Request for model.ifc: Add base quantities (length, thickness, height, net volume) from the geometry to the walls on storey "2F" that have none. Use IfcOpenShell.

First a look at what the model holds.

```python
import ifcopenshell
import ifcopenshell.util.element
import ifcopenshell.util.unit

model = ifcopenshell.open("model.ifc")
print(model.schema)
for unit_type in ("LENGTHUNIT", "AREAUNIT", "VOLUMEUNIT"):
    print(unit_type, ifcopenshell.util.unit.calculate_unit_scale(model, unit_type))
storey = next(s for s in model.by_type("IfcBuildingStorey") if s.Name == "2F")
walls = [e for e in ifcopenshell.util.element.get_decomposition(storey) if e.is_a("IfcWall")]
for e in sorted(walls, key=lambda e: e.id()):
    print(e.id(), e.is_a(), e.Name, list(ifcopenshell.util.element.get_psets(e, qtos_only=True)), sep=" | ")
```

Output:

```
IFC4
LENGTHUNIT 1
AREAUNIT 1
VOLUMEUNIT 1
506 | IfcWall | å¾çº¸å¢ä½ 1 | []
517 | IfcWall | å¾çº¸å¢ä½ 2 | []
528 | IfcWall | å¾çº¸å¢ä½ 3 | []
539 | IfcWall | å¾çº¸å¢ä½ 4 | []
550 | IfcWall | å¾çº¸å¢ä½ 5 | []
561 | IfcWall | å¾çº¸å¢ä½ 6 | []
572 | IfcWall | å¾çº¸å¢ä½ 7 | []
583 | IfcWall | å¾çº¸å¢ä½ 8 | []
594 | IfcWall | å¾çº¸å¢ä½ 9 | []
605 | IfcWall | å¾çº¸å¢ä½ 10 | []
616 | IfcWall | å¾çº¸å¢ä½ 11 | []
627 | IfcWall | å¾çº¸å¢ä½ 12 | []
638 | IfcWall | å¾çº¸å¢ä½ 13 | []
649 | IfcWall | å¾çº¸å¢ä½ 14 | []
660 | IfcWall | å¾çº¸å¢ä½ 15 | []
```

```python
import ifcopenshell
import ifcopenshell.api.pset
import ifcopenshell.geom
import ifcopenshell.util.element
import ifcopenshell.util.shape
import ifcopenshell.util.unit

model = ifcopenshell.open("model.ifc")
unit_scale = ifcopenshell.util.unit.calculate_unit_scale(model)
volume_scale = ifcopenshell.util.unit.calculate_unit_scale(model, "VOLUMEUNIT")
settings = ifcopenshell.geom.settings()

storey = next(s for s in model.by_type("IfcBuildingStorey") if s.Name == "2F")
walls = [e for e in ifcopenshell.util.element.get_decomposition(storey) if e.is_a("IfcWall")]

for e in sorted(walls, key=lambda e: e.id()):
    if ifcopenshell.util.element.get_psets(e, qtos_only=True, should_inherit=False):
        continue
    # Geometry comes back in metres, in the element's own axes.
    shape = ifcopenshell.geom.create_shape(settings, e)
    values = {
        "Length": ifcopenshell.util.shape.get_x(shape.geometry) / unit_scale,
        "Width": ifcopenshell.util.shape.get_y(shape.geometry) / unit_scale,
        "Height": ifcopenshell.util.shape.get_z(shape.geometry) / unit_scale,
        "NetVolume": ifcopenshell.util.shape.get_volume(shape.geometry) / volume_scale,
    }
    qto = ifcopenshell.api.pset.add_qto(model, product=e, name="Qto_WallBaseQuantities")
    ifcopenshell.api.pset.edit_qto(model, qto=qto, properties=values)
    print(e.id(), {k: round(v, 3) for k, v in values.items()})

model.write("model_v2.ifc")
```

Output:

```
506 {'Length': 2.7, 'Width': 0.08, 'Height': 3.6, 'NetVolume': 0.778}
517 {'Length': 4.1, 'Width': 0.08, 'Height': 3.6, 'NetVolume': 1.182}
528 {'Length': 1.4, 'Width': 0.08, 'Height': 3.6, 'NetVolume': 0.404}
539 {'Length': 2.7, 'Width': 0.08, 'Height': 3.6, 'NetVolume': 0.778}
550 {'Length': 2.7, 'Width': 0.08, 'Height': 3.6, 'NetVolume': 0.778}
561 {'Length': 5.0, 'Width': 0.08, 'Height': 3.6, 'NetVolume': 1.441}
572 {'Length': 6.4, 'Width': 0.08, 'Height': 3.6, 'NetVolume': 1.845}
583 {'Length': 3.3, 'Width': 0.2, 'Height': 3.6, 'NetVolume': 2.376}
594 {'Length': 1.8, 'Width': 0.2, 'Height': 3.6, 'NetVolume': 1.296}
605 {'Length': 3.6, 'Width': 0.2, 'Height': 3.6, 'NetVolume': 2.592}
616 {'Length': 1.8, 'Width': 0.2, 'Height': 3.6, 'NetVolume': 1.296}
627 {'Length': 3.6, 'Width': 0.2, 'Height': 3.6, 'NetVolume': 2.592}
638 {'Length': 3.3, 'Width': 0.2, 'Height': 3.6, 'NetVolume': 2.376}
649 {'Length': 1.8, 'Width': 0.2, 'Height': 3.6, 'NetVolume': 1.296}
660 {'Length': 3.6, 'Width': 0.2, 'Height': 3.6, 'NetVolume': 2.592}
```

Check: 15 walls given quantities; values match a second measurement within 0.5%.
